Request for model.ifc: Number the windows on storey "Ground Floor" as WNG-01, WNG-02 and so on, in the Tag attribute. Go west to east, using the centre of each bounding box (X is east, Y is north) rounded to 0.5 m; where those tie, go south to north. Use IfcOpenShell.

First a look at what the model holds.

```python
import ifcopenshell
import ifcopenshell.util.element
import ifcopenshell.util.placement

model = ifcopenshell.open("model.ifc")
print(model.schema)
storey = next(s for s in model.by_type("IfcBuildingStorey") if s.Name == "Ground Floor")
windows = [e for e in ifcopenshell.util.element.get_decomposition(storey) if e.is_a("IfcWindow")]
for e in sorted(windows, key=lambda e: e.id()):
    origin = ifcopenshell.util.placement.get_local_placement(e.ObjectPlacement)[:3, 3]
    print(e.id(), e.Tag, e.Name, origin.round(2) + 0.0, sep=" | ")
```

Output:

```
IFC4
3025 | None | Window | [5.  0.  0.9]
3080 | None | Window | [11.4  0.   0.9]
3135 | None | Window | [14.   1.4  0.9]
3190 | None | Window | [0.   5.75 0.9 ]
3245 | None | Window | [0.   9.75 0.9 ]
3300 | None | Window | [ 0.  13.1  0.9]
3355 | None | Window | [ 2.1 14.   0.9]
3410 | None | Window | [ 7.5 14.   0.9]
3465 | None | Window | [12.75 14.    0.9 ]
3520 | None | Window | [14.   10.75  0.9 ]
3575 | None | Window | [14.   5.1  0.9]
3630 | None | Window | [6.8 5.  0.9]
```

```python
import ifcopenshell
import ifcopenshell.geom
import ifcopenshell.util.element
import ifcopenshell.util.shape

model = ifcopenshell.open("model.ifc")
settings = ifcopenshell.geom.settings()
settings.set("use-world-coords", True)


def centre(element):
    shape = ifcopenshell.geom.create_shape(settings, element)
    return ifcopenshell.util.shape.get_bbox_centroid(shape.geometry)


storey = next(s for s in model.by_type("IfcBuildingStorey") if s.Name == "Ground Floor")
windows = [e for e in ifcopenshell.util.element.get_decomposition(storey) if e.is_a("IfcWindow")]

# Insertion points can sit at a corner or the storey origin, so sort by the geometry (in metres).
centres = {e: centre(e) for e in windows}
windows.sort(key=lambda e: (round(centres[e][0] / 0.5), centres[e][1]))

for i, e in enumerate(windows, start=1):
    number = f"WNG-{i:02d}"
    e.Tag = number
    print(e.id(), number)

model.write("model_v2.ifc")
```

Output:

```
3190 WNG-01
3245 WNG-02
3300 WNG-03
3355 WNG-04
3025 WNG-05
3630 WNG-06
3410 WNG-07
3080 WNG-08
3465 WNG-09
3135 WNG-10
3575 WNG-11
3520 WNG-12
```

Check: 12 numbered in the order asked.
